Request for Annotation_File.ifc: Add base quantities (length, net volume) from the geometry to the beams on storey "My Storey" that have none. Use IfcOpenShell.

First a look at what the model holds.

```python
import ifcopenshell
import ifcopenshell.util.element
import ifcopenshell.util.unit

model = ifcopenshell.open("Annotation_File.ifc")
print(model.schema)
for unit_type in ("LENGTHUNIT", "AREAUNIT", "VOLUMEUNIT"):
    print(unit_type, ifcopenshell.util.unit.calculate_unit_scale(model, unit_type))
storey = next(s for s in model.by_type("IfcBuildingStorey") if s.Name == "My Storey")
beams = [e for e in ifcopenshell.util.element.get_decomposition(storey) if e.is_a("IfcBeam")]
for e in sorted(beams, key=lambda e: e.id()):
    print(e.id(), e.is_a(), e.Name, list(ifcopenshell.util.element.get_psets(e, qtos_only=True)), sep=" | ")
```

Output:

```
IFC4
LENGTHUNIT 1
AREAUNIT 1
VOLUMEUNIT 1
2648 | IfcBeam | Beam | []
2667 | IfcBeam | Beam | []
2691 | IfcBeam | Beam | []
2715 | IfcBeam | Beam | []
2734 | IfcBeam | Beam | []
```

```python
import ifcopenshell
import ifcopenshell.api.pset
import ifcopenshell.geom
import ifcopenshell.util.element
import ifcopenshell.util.shape
import ifcopenshell.util.unit

model = ifcopenshell.open("Annotation_File.ifc")
unit_scale = ifcopenshell.util.unit.calculate_unit_scale(model)
volume_scale = ifcopenshell.util.unit.calculate_unit_scale(model, "VOLUMEUNIT")
settings = ifcopenshell.geom.settings()

storey = next(s for s in model.by_type("IfcBuildingStorey") if s.Name == "My Storey")
beams = [e for e in ifcopenshell.util.element.get_decomposition(storey) if e.is_a("IfcBeam")]

for e in sorted(beams, key=lambda e: e.id()):
    if ifcopenshell.util.element.get_psets(e, qtos_only=True, should_inherit=False):
        continue
    # Geometry comes back in metres, in the element's own axes.
    shape = ifcopenshell.geom.create_shape(settings, e)
    values = {
        "Length": ifcopenshell.util.shape.get_max_xyz(shape.geometry) / unit_scale,
        "NetVolume": ifcopenshell.util.shape.get_volume(shape.geometry) / volume_scale,
    }
    qto = ifcopenshell.api.pset.add_qto(model, product=e, name="Qto_BeamBaseQuantities")
    ifcopenshell.api.pset.edit_qto(model, qto=qto, properties=values)
    print(e.id(), {k: round(v, 3) for k, v in values.items()})

model.write("Annotation_File_v2.ifc")
```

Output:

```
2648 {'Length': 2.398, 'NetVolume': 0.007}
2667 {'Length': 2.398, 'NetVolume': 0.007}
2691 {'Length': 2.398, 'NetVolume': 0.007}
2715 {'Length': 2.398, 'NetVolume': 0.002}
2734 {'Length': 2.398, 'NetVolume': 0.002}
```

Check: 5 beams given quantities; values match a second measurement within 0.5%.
